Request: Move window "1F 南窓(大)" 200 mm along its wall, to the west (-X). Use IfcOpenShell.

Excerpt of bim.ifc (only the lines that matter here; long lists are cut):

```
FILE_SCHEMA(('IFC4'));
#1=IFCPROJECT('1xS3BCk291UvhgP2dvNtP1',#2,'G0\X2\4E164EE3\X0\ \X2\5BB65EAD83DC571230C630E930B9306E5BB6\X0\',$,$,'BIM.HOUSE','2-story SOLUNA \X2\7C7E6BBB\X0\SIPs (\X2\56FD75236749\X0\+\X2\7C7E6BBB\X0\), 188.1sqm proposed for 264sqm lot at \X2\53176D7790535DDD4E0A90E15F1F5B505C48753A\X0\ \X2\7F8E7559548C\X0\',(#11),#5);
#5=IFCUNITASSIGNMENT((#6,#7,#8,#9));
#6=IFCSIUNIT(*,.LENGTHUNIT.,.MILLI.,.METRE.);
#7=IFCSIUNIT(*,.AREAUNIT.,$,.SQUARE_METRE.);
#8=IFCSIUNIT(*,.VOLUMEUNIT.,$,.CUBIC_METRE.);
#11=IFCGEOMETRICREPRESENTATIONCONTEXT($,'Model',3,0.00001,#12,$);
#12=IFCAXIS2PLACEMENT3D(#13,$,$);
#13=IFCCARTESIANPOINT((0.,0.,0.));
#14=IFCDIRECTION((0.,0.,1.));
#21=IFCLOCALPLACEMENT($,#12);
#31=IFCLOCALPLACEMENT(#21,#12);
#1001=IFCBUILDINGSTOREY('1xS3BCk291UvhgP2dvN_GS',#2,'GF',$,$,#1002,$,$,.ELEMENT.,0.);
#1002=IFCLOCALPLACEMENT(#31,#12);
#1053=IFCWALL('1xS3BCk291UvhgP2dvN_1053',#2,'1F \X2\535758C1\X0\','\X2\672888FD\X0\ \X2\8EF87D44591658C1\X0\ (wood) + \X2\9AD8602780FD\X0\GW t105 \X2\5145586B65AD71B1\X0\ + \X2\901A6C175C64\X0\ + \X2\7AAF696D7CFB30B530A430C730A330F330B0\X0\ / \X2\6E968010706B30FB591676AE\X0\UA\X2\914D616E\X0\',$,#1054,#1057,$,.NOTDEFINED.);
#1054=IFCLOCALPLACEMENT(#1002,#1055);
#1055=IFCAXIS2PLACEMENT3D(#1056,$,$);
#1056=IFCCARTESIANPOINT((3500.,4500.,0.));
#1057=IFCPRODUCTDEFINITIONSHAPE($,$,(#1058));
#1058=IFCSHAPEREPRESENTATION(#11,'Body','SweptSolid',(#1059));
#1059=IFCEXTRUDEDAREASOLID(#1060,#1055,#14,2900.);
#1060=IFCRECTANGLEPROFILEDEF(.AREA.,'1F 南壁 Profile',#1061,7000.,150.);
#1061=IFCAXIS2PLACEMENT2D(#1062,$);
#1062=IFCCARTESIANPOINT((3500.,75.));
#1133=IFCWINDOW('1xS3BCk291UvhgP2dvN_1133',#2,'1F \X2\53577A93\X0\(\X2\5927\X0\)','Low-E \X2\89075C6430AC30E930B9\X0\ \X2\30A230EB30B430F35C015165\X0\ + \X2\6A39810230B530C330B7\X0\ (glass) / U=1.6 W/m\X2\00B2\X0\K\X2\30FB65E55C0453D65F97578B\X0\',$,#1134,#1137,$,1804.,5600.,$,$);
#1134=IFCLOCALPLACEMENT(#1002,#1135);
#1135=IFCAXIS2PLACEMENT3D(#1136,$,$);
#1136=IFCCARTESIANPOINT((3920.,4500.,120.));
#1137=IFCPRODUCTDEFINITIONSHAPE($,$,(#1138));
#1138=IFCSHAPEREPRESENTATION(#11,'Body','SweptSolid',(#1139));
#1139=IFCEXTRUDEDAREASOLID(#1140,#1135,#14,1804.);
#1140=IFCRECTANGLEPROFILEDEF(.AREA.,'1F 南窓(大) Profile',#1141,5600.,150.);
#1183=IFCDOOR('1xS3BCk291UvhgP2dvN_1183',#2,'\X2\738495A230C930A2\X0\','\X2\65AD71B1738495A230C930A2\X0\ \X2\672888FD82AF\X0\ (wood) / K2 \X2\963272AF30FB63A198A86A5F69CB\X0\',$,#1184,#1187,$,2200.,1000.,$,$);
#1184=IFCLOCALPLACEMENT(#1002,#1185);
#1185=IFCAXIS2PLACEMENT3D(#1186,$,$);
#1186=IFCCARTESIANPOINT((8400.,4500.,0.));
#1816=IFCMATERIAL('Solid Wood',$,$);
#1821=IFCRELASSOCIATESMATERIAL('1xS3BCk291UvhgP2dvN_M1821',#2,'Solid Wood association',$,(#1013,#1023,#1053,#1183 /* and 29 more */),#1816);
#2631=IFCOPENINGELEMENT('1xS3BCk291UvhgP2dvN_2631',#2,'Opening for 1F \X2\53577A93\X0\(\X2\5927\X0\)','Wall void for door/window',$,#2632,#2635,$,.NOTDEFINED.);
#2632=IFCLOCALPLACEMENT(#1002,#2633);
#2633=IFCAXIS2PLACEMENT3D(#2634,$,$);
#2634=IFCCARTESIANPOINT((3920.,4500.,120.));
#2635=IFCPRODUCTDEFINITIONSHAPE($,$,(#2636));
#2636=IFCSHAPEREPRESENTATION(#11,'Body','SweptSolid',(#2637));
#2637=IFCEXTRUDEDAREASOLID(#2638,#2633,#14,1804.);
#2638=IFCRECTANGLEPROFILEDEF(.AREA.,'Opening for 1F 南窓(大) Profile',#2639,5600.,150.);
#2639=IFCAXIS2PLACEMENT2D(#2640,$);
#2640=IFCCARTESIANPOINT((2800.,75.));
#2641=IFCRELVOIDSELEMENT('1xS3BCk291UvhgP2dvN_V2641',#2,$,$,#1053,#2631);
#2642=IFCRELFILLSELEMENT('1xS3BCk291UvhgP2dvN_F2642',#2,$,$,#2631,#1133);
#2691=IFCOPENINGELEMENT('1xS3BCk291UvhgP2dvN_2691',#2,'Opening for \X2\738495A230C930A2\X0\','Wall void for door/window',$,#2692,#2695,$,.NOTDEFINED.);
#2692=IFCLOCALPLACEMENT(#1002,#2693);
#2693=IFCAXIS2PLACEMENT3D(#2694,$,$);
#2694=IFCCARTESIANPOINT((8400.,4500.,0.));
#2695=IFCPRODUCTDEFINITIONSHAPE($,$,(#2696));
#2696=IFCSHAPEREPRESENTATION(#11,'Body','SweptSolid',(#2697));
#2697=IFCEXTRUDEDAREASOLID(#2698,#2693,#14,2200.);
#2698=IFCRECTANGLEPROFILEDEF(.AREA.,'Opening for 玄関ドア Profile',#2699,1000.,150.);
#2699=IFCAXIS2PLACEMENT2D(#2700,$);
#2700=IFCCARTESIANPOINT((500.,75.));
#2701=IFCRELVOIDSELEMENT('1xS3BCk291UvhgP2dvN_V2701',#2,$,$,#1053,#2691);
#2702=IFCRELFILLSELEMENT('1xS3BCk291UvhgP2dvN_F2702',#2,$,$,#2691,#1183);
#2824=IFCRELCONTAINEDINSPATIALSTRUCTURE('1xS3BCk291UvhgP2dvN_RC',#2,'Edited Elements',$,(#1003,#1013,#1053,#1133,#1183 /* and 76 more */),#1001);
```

```python
import ifcopenshell
import ifcopenshell.api.geometry
import ifcopenshell.util.placement
import ifcopenshell.util.unit

model = ifcopenshell.open("bim.ifc")
unit_scale = ifcopenshell.util.unit.calculate_unit_scale(model)

window = model.by_id(1133)
opening = window.FillsVoids[0].RelatingOpeningElement
wall = opening.VoidsElements[0].RelatingBuildingElement

wall_matrix = ifcopenshell.util.placement.get_local_placement(wall.ObjectPlacement)
shift = wall_matrix[:3, 0] * -0.2 / unit_scale
before = ifcopenshell.util.placement.get_local_placement(window.ObjectPlacement)[:3, 3].copy()

# The window is not placed relative to its opening, so move both.
for product in (opening, window):
    matrix = ifcopenshell.util.placement.get_local_placement(product.ObjectPlacement)
    matrix[:3, 3] += shift
    ifcopenshell.api.geometry.edit_object_placement(model, product=product, matrix=matrix, is_si=False)

after = ifcopenshell.util.placement.get_local_placement(window.ObjectPlacement)[:3, 3]
print("window moved by", (after - before).round(3) + 0.0)

model.write("bim_updated.ifc")
```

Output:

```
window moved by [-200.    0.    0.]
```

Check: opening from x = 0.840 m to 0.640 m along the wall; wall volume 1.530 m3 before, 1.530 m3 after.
